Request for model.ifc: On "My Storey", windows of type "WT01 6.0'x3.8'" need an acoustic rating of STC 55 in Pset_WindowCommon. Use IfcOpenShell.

First a look at what the model holds.

```python
import ifcopenshell
import ifcopenshell.util.element

model = ifcopenshell.open("model.ifc")
print(model.schema)
storey = next(s for s in model.by_type("IfcBuildingStorey") if s.Name == "My Storey")
windows = [e for e in ifcopenshell.util.element.get_decomposition(storey) if e.is_a("IfcWindow")]
seen = {}
for e in windows:
    element_type = ifcopenshell.util.element.get_type(e)
    key = (element_type.Name if element_type != e and element_type else None, ifcopenshell.util.element.get_pset(e, "Pset_WindowCommon", "AcousticRating"))
    seen[key] = seen.get(key, 0) + 1
for (name, value), count in sorted(seen.items(), key=str):
    print(count, "x", name, "|", value)
```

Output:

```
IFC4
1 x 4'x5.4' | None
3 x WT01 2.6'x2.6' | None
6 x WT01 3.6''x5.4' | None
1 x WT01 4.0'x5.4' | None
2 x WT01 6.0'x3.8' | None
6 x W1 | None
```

```python
import ifcopenshell
import ifcopenshell.api.pset
import ifcopenshell.util.element

model = ifcopenshell.open("model.ifc")

storey = next(s for s in model.by_type("IfcBuildingStorey") if s.Name == "My Storey")
windows = [e for e in ifcopenshell.util.element.get_decomposition(storey) if e.is_a("IfcWindow")]

count = 0
for e in windows:
    element_type = ifcopenshell.util.element.get_type(e)
    if element_type in (None, e) or element_type.Name != "WT01 6.0'x3.8'":
        continue
    # add_pset returns the element's existing set when there is one.
    pset = ifcopenshell.api.pset.add_pset(model, product=e, name="Pset_WindowCommon")
    ifcopenshell.api.pset.edit_pset(model, pset=pset, properties={"AcousticRating": "STC 55"})
    count += 1

print(count, "windows updated")

model.write("model-out.ifc")
```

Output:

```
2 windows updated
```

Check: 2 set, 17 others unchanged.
